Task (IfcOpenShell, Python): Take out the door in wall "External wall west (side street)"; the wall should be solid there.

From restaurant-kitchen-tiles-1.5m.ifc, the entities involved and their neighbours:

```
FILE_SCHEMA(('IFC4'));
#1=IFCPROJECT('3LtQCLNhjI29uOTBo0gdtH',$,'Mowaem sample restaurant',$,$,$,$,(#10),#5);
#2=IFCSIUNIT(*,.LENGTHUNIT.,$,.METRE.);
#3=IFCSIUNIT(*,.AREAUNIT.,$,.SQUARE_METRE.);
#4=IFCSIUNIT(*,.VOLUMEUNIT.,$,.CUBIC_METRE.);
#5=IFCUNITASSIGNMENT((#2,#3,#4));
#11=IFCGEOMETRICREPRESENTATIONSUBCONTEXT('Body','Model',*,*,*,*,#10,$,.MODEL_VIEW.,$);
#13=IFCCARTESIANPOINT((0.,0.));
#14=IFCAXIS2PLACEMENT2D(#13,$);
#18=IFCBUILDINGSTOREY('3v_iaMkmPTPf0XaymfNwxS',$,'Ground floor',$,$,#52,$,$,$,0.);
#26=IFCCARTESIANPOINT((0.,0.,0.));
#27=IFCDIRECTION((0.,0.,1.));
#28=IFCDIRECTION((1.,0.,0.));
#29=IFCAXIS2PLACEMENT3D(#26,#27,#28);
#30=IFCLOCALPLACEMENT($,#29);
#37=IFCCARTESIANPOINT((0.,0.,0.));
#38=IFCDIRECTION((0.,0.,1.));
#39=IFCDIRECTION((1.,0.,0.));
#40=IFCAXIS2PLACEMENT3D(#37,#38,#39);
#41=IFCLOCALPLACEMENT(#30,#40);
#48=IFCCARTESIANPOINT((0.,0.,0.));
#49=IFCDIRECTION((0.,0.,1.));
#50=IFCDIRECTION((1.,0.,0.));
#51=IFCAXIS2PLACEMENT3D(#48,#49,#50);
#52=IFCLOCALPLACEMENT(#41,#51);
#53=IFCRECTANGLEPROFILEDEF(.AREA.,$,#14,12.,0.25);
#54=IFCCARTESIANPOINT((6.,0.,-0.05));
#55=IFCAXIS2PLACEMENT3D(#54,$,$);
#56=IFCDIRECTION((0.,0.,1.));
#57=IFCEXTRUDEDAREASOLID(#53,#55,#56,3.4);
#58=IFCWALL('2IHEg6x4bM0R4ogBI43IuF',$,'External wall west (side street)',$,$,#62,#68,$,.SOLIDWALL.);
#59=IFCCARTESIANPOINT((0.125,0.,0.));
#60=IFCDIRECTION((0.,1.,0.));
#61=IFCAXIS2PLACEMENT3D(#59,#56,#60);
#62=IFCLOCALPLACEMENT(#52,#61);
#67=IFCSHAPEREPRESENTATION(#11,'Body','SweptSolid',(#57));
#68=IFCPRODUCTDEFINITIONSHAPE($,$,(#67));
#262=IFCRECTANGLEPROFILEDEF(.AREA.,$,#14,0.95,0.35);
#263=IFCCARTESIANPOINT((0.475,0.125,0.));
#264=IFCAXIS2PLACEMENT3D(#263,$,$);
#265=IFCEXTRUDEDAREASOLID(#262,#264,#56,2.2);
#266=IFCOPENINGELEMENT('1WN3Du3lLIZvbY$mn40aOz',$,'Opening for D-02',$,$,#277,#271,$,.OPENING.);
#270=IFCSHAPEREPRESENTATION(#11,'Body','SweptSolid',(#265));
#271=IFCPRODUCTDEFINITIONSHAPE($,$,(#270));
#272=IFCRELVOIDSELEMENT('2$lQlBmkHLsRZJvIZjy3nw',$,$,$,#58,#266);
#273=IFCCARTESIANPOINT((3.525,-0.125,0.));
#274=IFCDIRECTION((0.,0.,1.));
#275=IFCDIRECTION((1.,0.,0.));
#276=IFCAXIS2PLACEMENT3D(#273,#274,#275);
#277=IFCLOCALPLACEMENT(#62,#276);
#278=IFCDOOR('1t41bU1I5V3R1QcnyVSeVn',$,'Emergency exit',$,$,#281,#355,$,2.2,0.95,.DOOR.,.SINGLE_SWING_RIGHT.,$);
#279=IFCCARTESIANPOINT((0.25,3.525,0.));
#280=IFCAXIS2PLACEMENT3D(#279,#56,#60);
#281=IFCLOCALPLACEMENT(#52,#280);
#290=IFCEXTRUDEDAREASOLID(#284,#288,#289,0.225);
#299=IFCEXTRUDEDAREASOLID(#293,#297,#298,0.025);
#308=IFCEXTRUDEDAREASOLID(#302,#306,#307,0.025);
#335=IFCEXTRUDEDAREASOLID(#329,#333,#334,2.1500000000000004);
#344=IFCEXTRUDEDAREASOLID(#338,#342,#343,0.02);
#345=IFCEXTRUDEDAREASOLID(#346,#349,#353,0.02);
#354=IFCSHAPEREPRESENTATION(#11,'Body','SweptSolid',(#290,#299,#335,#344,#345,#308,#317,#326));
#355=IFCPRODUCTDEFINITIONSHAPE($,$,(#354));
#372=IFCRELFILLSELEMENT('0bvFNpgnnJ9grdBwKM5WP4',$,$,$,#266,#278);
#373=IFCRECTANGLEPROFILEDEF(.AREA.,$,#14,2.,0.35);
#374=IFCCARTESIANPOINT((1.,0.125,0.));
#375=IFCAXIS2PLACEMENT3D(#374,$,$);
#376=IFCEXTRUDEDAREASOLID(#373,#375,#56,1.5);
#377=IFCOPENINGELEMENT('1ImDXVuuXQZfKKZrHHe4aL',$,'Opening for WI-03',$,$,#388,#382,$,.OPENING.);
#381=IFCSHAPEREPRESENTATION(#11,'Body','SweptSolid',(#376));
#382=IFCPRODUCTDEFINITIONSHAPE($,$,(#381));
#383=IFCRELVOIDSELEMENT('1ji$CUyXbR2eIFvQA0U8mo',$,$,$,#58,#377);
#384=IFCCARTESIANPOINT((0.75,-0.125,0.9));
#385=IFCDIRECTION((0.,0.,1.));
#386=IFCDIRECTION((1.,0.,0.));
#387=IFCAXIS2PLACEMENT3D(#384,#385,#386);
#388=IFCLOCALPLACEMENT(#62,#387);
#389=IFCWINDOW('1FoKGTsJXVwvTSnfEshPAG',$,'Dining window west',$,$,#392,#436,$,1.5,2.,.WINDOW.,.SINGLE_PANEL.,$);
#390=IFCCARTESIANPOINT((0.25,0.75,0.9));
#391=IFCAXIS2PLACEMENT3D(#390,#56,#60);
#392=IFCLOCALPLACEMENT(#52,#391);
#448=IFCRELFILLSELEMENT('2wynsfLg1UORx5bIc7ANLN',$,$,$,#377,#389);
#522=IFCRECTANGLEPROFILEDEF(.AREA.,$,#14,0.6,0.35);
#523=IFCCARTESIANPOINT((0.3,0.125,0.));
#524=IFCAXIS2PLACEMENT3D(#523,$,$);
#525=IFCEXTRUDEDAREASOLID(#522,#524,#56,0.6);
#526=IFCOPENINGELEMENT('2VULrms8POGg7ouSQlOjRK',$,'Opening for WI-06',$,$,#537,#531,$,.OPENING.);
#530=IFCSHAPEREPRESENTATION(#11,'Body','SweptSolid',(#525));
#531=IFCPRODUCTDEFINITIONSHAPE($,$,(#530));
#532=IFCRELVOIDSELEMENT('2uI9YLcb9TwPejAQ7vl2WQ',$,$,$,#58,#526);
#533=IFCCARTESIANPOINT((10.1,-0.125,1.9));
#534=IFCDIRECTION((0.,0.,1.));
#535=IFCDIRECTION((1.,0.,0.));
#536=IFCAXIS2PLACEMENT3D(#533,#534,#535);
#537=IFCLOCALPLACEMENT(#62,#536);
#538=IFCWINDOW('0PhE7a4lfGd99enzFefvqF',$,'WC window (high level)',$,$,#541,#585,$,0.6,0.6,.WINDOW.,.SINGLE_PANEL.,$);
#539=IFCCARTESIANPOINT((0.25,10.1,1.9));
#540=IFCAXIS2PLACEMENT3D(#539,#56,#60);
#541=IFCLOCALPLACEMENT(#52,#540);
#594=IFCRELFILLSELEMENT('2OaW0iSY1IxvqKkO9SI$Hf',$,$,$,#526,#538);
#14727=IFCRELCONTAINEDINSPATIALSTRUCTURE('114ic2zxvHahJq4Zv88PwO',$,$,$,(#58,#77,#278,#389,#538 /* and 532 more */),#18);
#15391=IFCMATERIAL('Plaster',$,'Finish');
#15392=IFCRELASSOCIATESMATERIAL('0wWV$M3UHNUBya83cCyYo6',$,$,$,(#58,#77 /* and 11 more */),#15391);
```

```python
import ifcopenshell
import ifcopenshell.api.feature
import ifcopenshell.api.root
import ifcopenshell.geom
import ifcopenshell.util.shape

model = ifcopenshell.open("restaurant-kitchen-tiles-1.5m.ifc")
settings = ifcopenshell.geom.settings()


def volume(element):
    """Net volume in cubic metres, openings subtracted."""
    shape = ifcopenshell.geom.create_shape(settings, element)
    return ifcopenshell.util.shape.get_volume(shape.geometry)


door = model.by_guid("1t41bU1I5V3R1QcnyVSeVn")
opening = door.FillsVoids[0].RelatingOpeningElement
wall = opening.VoidsElements[0].RelatingBuildingElement
before = volume(wall)

ifcopenshell.api.root.remove_product(model, product=door)
ifcopenshell.api.feature.remove_feature(model, feature=opening)

after = volume(wall)

print(f"wall volume {before:.3f} -> {after:.3f} m3")

model.write("restaurant-kitchen-tiles-1.5m_v2.ifc")
```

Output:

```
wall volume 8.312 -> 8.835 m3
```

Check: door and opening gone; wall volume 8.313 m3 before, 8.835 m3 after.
